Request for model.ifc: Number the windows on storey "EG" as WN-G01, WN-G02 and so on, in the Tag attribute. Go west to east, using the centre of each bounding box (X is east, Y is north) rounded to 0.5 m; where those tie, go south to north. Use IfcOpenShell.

First a look at what the model holds.

```python
import ifcopenshell
import ifcopenshell.util.element
import ifcopenshell.util.placement

model = ifcopenshell.open("model.ifc")
print(model.schema)
storey = next(s for s in model.by_type("IfcBuildingStorey") if s.Name == "EG")
windows = [e for e in ifcopenshell.util.element.get_decomposition(storey) if e.is_a("IfcWindow")]
for e in sorted(windows, key=lambda e: e.id()):
    origin = ifcopenshell.util.placement.get_local_placement(e.ObjectPlacement)[:3, 3]
    print(e.id(), e.Tag, e.Name, origin.round(2) + 0.0, sep=" | ")
```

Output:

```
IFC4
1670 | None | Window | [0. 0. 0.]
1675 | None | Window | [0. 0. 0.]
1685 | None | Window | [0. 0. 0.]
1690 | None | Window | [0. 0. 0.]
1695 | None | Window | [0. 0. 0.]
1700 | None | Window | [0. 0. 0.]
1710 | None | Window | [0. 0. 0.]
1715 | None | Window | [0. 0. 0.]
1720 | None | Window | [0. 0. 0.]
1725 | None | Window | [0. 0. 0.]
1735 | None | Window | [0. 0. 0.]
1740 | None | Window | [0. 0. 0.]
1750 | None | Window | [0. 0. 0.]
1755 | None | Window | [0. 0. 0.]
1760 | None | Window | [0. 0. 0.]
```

```python
import ifcopenshell
import ifcopenshell.geom
import ifcopenshell.util.element
import ifcopenshell.util.shape

model = ifcopenshell.open("model.ifc")
settings = ifcopenshell.geom.settings()
settings.set("use-world-coords", True)


def centre(element):
    shape = ifcopenshell.geom.create_shape(settings, element)
    return ifcopenshell.util.shape.get_bbox_centroid(shape.geometry)


storey = next(s for s in model.by_type("IfcBuildingStorey") if s.Name == "EG")
windows = [e for e in ifcopenshell.util.element.get_decomposition(storey) if e.is_a("IfcWindow")]

# Insertion points can sit at a corner or the storey origin, so sort by the geometry (in metres).
centres = {e: centre(e) for e in windows}
windows.sort(key=lambda e: (round(centres[e][0] / 0.5), centres[e][1]))

for i, e in enumerate(windows, start=1):
    number = f"WN-G{i:02d}"
    e.Tag = number
    print(e.id(), number)

model.write("model-out.ifc")
```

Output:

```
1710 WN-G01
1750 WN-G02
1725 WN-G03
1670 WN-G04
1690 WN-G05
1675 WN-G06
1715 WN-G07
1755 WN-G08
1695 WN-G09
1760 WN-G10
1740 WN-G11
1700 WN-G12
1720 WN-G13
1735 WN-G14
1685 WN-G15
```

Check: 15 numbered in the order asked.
